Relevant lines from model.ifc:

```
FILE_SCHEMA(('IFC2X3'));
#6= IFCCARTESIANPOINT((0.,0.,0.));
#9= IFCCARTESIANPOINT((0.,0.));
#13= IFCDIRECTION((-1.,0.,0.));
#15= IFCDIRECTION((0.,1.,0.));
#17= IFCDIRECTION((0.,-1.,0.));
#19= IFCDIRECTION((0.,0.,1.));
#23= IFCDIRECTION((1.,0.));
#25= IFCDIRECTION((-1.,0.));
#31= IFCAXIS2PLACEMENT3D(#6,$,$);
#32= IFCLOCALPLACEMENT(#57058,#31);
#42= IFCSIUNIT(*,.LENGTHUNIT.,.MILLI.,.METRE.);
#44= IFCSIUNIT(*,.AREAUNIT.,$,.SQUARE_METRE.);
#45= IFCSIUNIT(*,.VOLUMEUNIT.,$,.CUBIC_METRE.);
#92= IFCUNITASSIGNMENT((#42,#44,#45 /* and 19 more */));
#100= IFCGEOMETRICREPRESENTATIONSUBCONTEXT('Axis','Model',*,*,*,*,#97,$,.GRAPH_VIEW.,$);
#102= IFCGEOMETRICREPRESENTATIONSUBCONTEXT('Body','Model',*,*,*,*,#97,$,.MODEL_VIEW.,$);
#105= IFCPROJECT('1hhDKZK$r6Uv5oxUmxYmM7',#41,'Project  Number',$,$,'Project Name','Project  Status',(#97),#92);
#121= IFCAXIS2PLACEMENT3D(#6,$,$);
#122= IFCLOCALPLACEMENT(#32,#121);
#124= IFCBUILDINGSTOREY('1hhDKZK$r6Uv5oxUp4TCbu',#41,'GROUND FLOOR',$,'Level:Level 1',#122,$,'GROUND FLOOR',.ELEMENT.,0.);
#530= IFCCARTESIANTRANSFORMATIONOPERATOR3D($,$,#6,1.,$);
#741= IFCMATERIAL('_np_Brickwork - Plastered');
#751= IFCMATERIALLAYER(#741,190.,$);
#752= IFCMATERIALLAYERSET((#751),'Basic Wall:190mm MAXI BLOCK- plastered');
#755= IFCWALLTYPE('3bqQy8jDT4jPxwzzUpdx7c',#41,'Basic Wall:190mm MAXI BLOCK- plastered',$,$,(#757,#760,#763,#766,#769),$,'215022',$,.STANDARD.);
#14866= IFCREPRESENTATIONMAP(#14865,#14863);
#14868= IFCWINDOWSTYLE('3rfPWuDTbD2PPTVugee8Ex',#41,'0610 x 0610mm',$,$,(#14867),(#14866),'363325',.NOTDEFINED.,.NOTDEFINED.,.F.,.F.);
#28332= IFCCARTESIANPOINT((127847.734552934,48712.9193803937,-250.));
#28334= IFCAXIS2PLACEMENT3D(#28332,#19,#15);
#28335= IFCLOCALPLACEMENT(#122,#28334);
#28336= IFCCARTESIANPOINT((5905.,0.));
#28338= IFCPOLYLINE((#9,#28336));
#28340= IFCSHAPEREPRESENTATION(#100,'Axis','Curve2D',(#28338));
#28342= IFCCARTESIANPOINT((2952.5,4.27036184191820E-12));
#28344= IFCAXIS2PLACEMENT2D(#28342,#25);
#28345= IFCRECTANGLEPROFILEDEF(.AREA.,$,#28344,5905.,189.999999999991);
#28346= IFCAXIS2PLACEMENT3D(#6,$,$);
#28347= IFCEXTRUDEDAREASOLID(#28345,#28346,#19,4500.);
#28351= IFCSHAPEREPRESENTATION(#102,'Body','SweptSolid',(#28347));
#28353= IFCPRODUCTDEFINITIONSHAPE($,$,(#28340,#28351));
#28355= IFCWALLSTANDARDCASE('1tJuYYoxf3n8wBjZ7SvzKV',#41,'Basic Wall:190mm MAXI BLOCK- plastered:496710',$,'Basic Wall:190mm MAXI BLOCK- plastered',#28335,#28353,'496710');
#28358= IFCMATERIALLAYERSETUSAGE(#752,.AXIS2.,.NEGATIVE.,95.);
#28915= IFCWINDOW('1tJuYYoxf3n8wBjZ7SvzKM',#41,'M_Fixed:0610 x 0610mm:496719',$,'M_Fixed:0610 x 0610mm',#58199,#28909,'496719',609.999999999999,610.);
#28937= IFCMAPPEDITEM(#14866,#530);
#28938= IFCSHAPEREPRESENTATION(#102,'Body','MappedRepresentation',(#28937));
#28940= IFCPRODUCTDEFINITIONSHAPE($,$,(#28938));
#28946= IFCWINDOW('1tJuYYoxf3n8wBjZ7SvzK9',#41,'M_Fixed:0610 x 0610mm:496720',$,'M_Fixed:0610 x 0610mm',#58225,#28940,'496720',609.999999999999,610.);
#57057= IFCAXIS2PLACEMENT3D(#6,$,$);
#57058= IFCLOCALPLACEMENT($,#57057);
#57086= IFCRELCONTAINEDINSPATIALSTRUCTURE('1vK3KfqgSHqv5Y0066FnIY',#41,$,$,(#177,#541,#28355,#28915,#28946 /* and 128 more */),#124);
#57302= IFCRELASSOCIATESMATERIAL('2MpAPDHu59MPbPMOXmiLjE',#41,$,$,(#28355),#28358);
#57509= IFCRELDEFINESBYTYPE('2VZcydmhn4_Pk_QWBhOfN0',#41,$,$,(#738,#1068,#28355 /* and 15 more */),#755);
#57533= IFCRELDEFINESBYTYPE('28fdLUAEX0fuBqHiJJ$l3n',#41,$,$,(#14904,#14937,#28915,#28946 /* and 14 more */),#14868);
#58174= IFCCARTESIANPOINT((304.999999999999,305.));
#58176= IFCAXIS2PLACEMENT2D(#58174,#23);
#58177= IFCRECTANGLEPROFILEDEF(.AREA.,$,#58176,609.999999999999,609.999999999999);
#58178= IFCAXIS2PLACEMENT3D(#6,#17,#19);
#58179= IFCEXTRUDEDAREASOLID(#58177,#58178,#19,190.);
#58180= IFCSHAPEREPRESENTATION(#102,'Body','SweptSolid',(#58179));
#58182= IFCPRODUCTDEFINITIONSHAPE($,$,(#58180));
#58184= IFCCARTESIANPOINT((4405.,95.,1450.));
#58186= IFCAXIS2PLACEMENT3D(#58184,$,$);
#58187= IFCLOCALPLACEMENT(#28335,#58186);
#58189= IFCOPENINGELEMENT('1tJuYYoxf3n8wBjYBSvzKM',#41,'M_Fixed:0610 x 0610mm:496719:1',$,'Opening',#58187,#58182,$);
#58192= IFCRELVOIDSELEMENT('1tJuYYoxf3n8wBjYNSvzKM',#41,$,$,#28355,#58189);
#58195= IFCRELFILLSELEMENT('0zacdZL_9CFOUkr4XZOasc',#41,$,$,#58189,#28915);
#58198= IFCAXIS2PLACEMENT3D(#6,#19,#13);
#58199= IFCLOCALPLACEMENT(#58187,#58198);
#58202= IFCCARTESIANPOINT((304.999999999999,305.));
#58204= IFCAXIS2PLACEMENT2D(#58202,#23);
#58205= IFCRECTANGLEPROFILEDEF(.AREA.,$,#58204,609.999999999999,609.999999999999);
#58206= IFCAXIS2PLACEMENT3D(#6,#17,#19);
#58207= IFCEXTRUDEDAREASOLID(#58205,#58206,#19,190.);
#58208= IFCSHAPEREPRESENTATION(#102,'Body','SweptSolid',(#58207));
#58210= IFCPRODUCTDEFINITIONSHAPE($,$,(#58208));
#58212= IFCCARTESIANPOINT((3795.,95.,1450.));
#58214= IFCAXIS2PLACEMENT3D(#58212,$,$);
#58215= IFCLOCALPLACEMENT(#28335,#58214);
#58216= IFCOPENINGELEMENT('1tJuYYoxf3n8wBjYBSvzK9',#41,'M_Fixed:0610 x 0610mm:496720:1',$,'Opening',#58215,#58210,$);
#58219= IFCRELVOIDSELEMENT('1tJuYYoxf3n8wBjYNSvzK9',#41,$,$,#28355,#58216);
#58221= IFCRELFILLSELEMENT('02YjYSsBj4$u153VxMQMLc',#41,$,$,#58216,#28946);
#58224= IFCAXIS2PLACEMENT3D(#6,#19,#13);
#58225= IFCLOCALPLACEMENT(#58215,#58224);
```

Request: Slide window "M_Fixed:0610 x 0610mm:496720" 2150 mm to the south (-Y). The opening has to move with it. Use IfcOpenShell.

```python
import ifcopenshell
import ifcopenshell.api.geometry
import ifcopenshell.util.placement

model = ifcopenshell.open("model.ifc")

window = model.by_guid("1tJuYYoxf3n8wBjZ7SvzK9")
opening = window.FillsVoids[0].RelatingOpeningElement
wall = opening.VoidsElements[0].RelatingBuildingElement

wall_matrix = ifcopenshell.util.placement.get_local_placement(wall.ObjectPlacement)
shift = wall_matrix[:3, 0] * -2150.0
before = ifcopenshell.util.placement.get_local_placement(window.ObjectPlacement)[:3, 3].copy()

# The window is placed relative to its opening, so it follows when the opening moves.
matrix = ifcopenshell.util.placement.get_local_placement(opening.ObjectPlacement)
matrix[:3, 3] += shift
ifcopenshell.api.geometry.edit_object_placement(
    model, product=opening, matrix=matrix, is_si=False, should_transform_children=True
)

after = ifcopenshell.util.placement.get_local_placement(window.ObjectPlacement)[:3, 3]
print("window moved by", (after - before).round(3) + 0.0)

model.write("model-out.ifc")
```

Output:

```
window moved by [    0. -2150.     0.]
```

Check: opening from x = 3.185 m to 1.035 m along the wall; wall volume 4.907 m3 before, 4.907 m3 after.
